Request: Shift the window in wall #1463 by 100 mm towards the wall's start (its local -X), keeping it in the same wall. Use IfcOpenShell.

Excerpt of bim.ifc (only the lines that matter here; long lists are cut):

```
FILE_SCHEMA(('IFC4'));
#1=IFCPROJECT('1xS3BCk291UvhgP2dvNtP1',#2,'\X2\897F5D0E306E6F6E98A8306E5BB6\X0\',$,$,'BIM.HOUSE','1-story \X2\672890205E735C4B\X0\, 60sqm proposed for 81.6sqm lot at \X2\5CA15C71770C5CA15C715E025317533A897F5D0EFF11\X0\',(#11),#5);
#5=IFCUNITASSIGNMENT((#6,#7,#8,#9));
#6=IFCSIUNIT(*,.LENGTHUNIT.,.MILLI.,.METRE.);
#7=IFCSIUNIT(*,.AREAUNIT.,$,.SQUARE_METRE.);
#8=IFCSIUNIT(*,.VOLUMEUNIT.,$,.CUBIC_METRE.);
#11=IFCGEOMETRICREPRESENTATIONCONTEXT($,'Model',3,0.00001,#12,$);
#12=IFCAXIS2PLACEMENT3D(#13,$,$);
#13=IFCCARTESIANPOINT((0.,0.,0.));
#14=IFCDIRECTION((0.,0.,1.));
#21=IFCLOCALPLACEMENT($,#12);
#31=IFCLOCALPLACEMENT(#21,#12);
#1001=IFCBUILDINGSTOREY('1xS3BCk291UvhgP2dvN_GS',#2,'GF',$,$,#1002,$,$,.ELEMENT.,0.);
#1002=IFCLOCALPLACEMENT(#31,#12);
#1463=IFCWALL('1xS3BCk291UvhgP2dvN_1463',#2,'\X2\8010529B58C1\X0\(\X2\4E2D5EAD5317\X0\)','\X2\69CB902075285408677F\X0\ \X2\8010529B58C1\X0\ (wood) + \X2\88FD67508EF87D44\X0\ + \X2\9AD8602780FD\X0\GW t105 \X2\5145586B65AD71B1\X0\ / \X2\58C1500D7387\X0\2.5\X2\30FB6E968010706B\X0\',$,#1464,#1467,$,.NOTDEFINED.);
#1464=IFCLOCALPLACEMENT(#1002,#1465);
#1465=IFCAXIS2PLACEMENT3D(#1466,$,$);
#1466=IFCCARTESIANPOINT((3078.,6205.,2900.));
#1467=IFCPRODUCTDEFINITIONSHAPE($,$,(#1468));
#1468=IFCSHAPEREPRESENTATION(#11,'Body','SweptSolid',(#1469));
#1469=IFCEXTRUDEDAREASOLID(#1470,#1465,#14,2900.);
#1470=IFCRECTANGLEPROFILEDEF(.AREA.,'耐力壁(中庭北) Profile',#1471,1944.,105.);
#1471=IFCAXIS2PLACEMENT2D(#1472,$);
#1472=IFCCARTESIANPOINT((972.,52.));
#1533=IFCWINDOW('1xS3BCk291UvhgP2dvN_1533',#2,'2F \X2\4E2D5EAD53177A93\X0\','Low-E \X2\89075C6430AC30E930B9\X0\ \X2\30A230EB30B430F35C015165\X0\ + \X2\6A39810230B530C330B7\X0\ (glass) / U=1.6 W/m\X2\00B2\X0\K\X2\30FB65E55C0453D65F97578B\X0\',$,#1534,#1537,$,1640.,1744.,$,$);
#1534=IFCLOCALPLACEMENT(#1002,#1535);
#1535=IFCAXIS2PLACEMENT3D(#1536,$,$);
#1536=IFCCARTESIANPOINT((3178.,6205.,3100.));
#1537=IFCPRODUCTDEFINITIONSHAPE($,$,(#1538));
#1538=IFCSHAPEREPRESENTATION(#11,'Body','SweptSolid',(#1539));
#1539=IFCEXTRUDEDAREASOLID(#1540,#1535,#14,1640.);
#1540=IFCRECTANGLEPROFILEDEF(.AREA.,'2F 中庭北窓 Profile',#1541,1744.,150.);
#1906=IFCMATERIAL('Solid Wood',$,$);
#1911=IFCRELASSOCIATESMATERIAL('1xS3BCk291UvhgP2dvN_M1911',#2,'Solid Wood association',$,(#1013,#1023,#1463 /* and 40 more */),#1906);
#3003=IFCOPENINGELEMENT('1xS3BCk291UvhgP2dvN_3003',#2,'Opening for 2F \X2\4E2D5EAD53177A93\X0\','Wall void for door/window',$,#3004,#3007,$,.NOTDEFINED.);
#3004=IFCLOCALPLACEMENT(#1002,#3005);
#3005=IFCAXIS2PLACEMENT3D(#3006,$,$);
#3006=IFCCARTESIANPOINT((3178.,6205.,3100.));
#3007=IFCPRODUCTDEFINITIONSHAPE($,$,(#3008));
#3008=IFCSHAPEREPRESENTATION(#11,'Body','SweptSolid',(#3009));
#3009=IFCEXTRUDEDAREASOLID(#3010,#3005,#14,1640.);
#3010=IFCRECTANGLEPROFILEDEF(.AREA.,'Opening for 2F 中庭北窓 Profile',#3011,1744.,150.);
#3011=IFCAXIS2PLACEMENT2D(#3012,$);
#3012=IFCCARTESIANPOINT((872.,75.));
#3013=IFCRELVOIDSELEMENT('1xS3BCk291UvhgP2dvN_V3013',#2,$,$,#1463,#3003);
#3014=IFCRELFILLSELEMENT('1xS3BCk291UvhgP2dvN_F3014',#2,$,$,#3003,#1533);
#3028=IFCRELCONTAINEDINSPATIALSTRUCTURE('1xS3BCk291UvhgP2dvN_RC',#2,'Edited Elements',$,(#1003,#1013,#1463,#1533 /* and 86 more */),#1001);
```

```python
import ifcopenshell
import ifcopenshell.api.geometry
import ifcopenshell.util.placement
import ifcopenshell.util.unit

model = ifcopenshell.open("bim.ifc")
unit_scale = ifcopenshell.util.unit.calculate_unit_scale(model)

window = model.by_id(1533)
opening = window.FillsVoids[0].RelatingOpeningElement
wall = opening.VoidsElements[0].RelatingBuildingElement

wall_matrix = ifcopenshell.util.placement.get_local_placement(wall.ObjectPlacement)
shift = wall_matrix[:3, 0] * -0.1 / unit_scale
before = ifcopenshell.util.placement.get_local_placement(window.ObjectPlacement)[:3, 3].copy()

# The window is not placed relative to its opening, so move both.
for product in (opening, window):
    matrix = ifcopenshell.util.placement.get_local_placement(product.ObjectPlacement)
    matrix[:3, 3] += shift
    ifcopenshell.api.geometry.edit_object_placement(model, product=product, matrix=matrix, is_si=False)

after = ifcopenshell.util.placement.get_local_placement(window.ObjectPlacement)[:3, 3]
print("window moved by", (after - before).round(3) + 0.0)

model.write("bim-out.ifc")
```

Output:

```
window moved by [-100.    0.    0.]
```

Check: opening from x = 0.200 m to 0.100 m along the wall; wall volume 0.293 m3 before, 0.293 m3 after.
